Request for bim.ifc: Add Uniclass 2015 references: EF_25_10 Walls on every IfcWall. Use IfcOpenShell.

First a look at what the model holds.

```python
import ifcopenshell

model = ifcopenshell.open("bim.ifc")
print(model.schema)
print("classifications:", [c.Name for c in model.by_type("IfcClassification")])
for ifc_class in ("IfcDoor", "IfcRoof", "IfcStair", "IfcWall", "IfcWindow"):
    print(ifc_class, len(model.by_type(ifc_class)))
```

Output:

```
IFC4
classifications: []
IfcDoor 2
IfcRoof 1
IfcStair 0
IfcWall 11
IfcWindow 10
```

```python
import ifcopenshell
import ifcopenshell.api.classification

model = ifcopenshell.open("bim.ifc")

system = ifcopenshell.api.classification.add_classification(model, classification="Uniclass 2015")

codes = {
    "IfcWall": ("EF_25_10", "Walls"),
}
for ifc_class, (code, name) in codes.items():
    products = model.by_type(ifc_class)
    ifcopenshell.api.classification.add_reference(
        model, products=products, classification=system, identification=code, name=name
    )
    print(code, len(products))

model.write("bim_updated.ifc")
```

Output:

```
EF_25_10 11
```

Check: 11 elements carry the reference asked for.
